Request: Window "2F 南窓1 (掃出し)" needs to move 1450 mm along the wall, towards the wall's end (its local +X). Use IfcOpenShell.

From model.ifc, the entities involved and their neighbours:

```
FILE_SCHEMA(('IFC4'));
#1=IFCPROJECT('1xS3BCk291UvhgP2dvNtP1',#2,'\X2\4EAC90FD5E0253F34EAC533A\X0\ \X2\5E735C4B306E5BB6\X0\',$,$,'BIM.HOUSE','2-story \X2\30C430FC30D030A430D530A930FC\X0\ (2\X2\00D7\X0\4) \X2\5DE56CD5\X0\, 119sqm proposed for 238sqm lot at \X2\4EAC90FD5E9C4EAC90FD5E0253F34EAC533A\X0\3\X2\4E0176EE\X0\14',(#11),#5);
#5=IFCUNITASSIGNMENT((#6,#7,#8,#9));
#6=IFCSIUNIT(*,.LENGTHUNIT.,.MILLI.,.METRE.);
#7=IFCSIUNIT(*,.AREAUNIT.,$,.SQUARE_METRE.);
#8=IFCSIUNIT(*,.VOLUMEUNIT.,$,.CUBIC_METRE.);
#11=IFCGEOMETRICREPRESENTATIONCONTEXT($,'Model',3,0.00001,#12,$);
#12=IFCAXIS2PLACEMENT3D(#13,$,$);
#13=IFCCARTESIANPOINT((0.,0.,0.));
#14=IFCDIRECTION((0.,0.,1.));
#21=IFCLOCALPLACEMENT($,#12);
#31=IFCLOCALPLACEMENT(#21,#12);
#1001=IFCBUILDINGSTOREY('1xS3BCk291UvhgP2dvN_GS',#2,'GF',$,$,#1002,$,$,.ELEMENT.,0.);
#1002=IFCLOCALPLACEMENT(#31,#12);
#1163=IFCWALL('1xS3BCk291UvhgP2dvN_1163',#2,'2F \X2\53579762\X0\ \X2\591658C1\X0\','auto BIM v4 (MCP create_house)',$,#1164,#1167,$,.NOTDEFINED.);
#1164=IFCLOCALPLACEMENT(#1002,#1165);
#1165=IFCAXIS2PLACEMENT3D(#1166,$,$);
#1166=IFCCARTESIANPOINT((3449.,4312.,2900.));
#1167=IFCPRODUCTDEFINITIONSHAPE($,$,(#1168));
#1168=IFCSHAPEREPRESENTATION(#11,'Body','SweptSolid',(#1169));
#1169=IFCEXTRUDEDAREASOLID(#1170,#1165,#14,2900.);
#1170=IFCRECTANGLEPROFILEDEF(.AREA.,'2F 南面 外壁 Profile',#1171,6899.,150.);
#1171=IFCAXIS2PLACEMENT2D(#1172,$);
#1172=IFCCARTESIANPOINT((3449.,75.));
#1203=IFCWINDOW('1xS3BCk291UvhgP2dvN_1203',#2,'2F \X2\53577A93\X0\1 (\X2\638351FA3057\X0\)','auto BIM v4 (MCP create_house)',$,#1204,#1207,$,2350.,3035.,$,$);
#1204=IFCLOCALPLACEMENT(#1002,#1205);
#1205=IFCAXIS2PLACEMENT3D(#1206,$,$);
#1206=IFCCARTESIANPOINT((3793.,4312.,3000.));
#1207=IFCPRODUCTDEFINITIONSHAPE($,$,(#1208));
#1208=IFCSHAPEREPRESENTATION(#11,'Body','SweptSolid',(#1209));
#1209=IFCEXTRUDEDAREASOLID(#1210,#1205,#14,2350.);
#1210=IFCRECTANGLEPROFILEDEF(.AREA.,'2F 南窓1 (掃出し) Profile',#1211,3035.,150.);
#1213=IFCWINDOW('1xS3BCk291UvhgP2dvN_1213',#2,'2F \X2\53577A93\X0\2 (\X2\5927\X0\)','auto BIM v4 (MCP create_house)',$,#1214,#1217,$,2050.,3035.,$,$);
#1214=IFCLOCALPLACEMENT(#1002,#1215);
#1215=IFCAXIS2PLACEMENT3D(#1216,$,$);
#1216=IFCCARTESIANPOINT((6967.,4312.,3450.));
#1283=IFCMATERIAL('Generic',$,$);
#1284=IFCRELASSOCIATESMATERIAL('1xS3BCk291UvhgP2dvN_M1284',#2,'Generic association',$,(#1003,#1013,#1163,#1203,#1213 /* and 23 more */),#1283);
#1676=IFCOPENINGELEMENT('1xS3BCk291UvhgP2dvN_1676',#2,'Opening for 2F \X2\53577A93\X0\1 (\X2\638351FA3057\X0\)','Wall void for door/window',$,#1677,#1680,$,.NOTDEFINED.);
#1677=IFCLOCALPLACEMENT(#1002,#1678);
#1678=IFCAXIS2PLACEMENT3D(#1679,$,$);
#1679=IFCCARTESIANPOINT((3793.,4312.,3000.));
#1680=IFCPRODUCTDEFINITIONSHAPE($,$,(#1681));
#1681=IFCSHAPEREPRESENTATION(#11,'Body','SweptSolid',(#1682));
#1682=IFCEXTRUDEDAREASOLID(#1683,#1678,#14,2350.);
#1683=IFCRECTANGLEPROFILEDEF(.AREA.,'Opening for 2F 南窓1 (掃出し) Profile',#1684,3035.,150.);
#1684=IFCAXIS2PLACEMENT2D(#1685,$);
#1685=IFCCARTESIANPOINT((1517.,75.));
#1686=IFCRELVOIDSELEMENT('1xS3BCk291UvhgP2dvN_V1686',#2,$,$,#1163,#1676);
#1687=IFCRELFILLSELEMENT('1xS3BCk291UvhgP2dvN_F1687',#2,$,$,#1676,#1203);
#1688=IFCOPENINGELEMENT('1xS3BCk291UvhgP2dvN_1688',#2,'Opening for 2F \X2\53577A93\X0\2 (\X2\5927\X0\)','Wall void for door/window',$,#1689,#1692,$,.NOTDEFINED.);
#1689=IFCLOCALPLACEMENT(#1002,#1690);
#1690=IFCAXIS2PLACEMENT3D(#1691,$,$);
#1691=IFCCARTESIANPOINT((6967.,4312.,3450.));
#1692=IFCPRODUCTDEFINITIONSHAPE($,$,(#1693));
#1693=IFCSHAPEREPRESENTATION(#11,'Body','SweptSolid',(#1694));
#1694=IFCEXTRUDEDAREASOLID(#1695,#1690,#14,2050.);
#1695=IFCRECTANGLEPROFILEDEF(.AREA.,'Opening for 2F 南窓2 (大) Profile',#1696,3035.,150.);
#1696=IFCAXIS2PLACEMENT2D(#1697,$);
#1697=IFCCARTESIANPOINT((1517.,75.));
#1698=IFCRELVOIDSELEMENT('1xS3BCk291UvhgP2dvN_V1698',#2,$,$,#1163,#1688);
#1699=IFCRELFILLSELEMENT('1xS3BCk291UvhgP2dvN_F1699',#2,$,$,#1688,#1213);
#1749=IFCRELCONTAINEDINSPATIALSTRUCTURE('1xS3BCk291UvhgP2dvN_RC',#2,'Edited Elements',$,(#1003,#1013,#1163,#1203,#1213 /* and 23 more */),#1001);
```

```python
import ifcopenshell
import ifcopenshell.api.geometry
import ifcopenshell.util.placement

model = ifcopenshell.open("model.ifc")

window = model.by_guid("1xS3BCk291UvhgP2dvN_1203")
opening = window.FillsVoids[0].RelatingOpeningElement
wall = opening.VoidsElements[0].RelatingBuildingElement

wall_matrix = ifcopenshell.util.placement.get_local_placement(wall.ObjectPlacement)
shift = wall_matrix[:3, 0] * 1450.0
before = ifcopenshell.util.placement.get_local_placement(window.ObjectPlacement)[:3, 3].copy()

# The window is not placed relative to its opening, so move both.
for product in (opening, window):
    matrix = ifcopenshell.util.placement.get_local_placement(product.ObjectPlacement)
    matrix[:3, 3] += shift
    ifcopenshell.api.geometry.edit_object_placement(model, product=product, matrix=matrix, is_si=False)

after = ifcopenshell.util.placement.get_local_placement(window.ObjectPlacement)[:3, 3]
print("window moved by", (after - before).round(3) + 0.0)

model.write("model_updated.ifc")
```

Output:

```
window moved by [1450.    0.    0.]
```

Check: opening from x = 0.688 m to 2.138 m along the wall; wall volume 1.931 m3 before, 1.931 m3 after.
